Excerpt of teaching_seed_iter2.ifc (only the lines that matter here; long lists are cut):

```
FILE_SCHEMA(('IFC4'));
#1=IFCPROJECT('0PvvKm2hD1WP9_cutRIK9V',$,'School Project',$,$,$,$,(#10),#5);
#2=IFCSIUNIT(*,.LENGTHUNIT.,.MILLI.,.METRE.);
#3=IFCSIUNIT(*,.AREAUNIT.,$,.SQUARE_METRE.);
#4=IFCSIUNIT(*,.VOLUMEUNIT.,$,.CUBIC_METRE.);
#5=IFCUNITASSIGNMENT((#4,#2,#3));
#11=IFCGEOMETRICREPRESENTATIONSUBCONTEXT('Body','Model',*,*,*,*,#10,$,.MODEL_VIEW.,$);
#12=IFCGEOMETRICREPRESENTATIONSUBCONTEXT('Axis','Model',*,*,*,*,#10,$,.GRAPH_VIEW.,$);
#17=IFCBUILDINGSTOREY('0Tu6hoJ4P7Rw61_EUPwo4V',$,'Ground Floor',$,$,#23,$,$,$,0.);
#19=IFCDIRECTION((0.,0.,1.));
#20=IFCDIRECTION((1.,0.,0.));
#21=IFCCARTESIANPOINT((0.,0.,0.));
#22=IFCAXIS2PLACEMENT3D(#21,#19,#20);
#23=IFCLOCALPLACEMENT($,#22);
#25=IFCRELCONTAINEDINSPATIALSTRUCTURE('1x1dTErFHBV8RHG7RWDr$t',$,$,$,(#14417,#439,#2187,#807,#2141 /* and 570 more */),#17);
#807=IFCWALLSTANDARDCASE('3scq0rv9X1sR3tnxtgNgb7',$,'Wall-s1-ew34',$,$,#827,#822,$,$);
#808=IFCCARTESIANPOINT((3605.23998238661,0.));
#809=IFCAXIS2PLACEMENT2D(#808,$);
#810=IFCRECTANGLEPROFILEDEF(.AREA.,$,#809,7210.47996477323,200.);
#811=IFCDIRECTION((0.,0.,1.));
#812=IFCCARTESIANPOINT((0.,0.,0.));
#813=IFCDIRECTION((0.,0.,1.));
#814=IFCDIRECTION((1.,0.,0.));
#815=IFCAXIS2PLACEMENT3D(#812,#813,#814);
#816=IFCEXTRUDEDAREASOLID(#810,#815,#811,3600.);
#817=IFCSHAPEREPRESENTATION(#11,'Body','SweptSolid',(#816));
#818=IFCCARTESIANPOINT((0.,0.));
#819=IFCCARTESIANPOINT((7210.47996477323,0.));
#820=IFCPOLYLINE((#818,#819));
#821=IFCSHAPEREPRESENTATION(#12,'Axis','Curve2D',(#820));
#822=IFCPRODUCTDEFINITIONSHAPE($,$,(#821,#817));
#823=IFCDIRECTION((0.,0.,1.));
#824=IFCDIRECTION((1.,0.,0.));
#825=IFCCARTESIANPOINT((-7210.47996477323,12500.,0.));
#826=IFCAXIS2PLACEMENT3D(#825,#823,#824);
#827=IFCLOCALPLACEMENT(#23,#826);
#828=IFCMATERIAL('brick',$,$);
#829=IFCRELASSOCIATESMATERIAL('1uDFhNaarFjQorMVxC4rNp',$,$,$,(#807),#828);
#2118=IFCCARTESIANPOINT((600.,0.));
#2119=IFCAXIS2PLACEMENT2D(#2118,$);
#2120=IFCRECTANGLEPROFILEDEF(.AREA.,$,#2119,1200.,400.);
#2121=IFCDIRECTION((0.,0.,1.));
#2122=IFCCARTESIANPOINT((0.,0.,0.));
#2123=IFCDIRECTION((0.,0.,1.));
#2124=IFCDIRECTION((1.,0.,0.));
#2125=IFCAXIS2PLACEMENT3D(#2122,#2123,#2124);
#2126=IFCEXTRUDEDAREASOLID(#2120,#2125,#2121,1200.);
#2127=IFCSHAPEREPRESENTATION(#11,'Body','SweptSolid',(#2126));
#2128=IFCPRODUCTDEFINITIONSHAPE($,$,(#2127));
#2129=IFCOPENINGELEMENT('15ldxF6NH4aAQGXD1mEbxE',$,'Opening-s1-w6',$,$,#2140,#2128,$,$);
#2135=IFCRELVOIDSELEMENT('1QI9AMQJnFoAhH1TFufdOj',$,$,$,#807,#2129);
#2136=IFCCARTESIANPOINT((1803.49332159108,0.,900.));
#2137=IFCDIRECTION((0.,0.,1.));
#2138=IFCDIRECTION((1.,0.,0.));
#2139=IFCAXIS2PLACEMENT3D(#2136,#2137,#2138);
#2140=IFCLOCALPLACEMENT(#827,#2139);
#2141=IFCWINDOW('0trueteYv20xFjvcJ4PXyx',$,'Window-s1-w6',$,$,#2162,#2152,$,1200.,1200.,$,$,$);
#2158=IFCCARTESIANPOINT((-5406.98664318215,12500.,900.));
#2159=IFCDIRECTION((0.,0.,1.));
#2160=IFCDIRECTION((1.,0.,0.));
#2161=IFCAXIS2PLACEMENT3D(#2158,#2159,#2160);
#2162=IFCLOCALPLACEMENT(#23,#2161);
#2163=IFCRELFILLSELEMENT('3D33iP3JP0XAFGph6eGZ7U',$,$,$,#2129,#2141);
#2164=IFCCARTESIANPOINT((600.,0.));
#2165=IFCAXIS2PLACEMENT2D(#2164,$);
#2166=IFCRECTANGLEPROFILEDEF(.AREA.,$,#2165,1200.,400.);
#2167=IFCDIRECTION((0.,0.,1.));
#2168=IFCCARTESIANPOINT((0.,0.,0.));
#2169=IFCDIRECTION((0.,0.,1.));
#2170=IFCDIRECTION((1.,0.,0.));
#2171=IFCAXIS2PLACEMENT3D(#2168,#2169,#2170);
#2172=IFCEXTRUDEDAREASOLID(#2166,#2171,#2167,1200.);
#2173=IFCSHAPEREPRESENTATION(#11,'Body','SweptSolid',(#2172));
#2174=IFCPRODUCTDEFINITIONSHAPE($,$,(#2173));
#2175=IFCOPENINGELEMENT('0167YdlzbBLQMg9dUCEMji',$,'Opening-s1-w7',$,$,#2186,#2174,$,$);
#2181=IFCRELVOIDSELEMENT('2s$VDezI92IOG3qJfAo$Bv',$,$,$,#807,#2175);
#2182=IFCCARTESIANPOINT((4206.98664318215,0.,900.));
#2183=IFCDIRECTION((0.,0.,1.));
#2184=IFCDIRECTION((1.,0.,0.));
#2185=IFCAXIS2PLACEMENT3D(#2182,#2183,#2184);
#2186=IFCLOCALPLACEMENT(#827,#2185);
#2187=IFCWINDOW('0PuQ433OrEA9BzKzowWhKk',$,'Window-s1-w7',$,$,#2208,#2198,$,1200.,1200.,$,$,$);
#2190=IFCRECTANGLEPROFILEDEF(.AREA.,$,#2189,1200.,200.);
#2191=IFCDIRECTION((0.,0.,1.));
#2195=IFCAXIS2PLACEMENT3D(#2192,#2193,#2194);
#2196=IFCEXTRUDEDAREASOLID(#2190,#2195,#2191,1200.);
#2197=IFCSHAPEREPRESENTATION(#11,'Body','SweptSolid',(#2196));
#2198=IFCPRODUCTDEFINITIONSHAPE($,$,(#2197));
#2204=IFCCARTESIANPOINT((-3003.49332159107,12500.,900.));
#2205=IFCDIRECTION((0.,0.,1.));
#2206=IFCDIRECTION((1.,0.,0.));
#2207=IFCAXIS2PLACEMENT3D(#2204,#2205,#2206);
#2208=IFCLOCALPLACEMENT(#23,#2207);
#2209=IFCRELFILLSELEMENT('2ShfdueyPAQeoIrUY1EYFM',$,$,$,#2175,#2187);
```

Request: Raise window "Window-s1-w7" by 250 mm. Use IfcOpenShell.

```python
import numpy as np
import ifcopenshell
import ifcopenshell.api.geometry
import ifcopenshell.util.placement
import ifcopenshell.util.unit

model = ifcopenshell.open("teaching_seed_iter2.ifc")
unit_scale = ifcopenshell.util.unit.calculate_unit_scale(model)

window = model.by_id(2187)
opening = window.FillsVoids[0].RelatingOpeningElement
dz = 0.25 / unit_scale

shift = np.array([0.0, 0.0, dz])
# The window is not placed relative to its opening, so move both.
for product in (opening, window):
    matrix = ifcopenshell.util.placement.get_local_placement(product.ObjectPlacement)
    matrix[:3, 3] += shift
    ifcopenshell.api.geometry.edit_object_placement(model, product=product, matrix=matrix, is_si=False)

print(f"moved by {dz * unit_scale:+.3f} m")

model.write("teaching_seed_iter2_edited.ifc")
```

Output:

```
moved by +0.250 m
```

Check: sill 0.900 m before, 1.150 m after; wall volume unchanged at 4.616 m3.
